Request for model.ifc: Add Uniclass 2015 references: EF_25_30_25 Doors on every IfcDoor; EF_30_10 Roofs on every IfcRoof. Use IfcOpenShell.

First a look at what the model holds.

```python
import ifcopenshell

model = ifcopenshell.open("model.ifc")
print(model.schema)
print("classifications:", [c.Name for c in model.by_type("IfcClassification")])
for ifc_class in ("IfcDoor", "IfcRoof", "IfcStair", "IfcWall", "IfcWindow"):
    print(ifc_class, len(model.by_type(ifc_class)))
```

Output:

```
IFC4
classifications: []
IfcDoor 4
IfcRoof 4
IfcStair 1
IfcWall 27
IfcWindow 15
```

```python
import ifcopenshell
import ifcopenshell.api.classification

model = ifcopenshell.open("model.ifc")

system = ifcopenshell.api.classification.add_classification(model, classification="Uniclass 2015")

codes = {
    "IfcDoor": ("EF_25_30_25", "Doors"),
    "IfcRoof": ("EF_30_10", "Roofs"),
}
for ifc_class, (code, name) in codes.items():
    products = model.by_type(ifc_class)
    ifcopenshell.api.classification.add_reference(
        model, products=products, classification=system, identification=code, name=name
    )
    print(code, len(products))

model.write("model_edited.ifc")
```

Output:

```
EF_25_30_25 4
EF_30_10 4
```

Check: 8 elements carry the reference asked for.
